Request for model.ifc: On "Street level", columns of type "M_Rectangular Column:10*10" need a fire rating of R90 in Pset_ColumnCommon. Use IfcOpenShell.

First a look at what the model holds.

```python
import ifcopenshell
import ifcopenshell.util.element

model = ifcopenshell.open("model.ifc")
print(model.schema)
storey = next(s for s in model.by_type("IfcBuildingStorey") if s.Name == "Street level")
columns = [e for e in ifcopenshell.util.element.get_decomposition(storey) if e.is_a("IfcColumn")]
seen = {}
for e in columns:
    element_type = ifcopenshell.util.element.get_type(e)
    key = (element_type.Name if element_type != e and element_type else None, ifcopenshell.util.element.get_pset(e, "Pset_ColumnCommon", "FireRating"))
    seen[key] = seen.get(key, 0) + 1
for (name, value), count in sorted(seen.items(), key=str):
    print(count, "x", name, "|", value)
```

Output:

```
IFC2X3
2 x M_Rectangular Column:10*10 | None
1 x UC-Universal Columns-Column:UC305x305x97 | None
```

```python
import ifcopenshell
import ifcopenshell.api.pset
import ifcopenshell.util.element

model = ifcopenshell.open("model.ifc")

storey = next(s for s in model.by_type("IfcBuildingStorey") if s.Name == "Street level")
columns = [e for e in ifcopenshell.util.element.get_decomposition(storey) if e.is_a("IfcColumn")]

count = 0
for e in columns:
    element_type = ifcopenshell.util.element.get_type(e)
    if element_type in (None, e) or element_type.Name != "M_Rectangular Column:10*10":
        continue
    # add_pset returns the element's existing set when there is one.
    pset = ifcopenshell.api.pset.add_pset(model, product=e, name="Pset_ColumnCommon")
    ifcopenshell.api.pset.edit_pset(model, pset=pset, properties={"FireRating": "R90"})
    count += 1

print(count, "columns updated")

model.write("model-out.ifc")
```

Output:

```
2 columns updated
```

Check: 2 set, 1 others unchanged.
